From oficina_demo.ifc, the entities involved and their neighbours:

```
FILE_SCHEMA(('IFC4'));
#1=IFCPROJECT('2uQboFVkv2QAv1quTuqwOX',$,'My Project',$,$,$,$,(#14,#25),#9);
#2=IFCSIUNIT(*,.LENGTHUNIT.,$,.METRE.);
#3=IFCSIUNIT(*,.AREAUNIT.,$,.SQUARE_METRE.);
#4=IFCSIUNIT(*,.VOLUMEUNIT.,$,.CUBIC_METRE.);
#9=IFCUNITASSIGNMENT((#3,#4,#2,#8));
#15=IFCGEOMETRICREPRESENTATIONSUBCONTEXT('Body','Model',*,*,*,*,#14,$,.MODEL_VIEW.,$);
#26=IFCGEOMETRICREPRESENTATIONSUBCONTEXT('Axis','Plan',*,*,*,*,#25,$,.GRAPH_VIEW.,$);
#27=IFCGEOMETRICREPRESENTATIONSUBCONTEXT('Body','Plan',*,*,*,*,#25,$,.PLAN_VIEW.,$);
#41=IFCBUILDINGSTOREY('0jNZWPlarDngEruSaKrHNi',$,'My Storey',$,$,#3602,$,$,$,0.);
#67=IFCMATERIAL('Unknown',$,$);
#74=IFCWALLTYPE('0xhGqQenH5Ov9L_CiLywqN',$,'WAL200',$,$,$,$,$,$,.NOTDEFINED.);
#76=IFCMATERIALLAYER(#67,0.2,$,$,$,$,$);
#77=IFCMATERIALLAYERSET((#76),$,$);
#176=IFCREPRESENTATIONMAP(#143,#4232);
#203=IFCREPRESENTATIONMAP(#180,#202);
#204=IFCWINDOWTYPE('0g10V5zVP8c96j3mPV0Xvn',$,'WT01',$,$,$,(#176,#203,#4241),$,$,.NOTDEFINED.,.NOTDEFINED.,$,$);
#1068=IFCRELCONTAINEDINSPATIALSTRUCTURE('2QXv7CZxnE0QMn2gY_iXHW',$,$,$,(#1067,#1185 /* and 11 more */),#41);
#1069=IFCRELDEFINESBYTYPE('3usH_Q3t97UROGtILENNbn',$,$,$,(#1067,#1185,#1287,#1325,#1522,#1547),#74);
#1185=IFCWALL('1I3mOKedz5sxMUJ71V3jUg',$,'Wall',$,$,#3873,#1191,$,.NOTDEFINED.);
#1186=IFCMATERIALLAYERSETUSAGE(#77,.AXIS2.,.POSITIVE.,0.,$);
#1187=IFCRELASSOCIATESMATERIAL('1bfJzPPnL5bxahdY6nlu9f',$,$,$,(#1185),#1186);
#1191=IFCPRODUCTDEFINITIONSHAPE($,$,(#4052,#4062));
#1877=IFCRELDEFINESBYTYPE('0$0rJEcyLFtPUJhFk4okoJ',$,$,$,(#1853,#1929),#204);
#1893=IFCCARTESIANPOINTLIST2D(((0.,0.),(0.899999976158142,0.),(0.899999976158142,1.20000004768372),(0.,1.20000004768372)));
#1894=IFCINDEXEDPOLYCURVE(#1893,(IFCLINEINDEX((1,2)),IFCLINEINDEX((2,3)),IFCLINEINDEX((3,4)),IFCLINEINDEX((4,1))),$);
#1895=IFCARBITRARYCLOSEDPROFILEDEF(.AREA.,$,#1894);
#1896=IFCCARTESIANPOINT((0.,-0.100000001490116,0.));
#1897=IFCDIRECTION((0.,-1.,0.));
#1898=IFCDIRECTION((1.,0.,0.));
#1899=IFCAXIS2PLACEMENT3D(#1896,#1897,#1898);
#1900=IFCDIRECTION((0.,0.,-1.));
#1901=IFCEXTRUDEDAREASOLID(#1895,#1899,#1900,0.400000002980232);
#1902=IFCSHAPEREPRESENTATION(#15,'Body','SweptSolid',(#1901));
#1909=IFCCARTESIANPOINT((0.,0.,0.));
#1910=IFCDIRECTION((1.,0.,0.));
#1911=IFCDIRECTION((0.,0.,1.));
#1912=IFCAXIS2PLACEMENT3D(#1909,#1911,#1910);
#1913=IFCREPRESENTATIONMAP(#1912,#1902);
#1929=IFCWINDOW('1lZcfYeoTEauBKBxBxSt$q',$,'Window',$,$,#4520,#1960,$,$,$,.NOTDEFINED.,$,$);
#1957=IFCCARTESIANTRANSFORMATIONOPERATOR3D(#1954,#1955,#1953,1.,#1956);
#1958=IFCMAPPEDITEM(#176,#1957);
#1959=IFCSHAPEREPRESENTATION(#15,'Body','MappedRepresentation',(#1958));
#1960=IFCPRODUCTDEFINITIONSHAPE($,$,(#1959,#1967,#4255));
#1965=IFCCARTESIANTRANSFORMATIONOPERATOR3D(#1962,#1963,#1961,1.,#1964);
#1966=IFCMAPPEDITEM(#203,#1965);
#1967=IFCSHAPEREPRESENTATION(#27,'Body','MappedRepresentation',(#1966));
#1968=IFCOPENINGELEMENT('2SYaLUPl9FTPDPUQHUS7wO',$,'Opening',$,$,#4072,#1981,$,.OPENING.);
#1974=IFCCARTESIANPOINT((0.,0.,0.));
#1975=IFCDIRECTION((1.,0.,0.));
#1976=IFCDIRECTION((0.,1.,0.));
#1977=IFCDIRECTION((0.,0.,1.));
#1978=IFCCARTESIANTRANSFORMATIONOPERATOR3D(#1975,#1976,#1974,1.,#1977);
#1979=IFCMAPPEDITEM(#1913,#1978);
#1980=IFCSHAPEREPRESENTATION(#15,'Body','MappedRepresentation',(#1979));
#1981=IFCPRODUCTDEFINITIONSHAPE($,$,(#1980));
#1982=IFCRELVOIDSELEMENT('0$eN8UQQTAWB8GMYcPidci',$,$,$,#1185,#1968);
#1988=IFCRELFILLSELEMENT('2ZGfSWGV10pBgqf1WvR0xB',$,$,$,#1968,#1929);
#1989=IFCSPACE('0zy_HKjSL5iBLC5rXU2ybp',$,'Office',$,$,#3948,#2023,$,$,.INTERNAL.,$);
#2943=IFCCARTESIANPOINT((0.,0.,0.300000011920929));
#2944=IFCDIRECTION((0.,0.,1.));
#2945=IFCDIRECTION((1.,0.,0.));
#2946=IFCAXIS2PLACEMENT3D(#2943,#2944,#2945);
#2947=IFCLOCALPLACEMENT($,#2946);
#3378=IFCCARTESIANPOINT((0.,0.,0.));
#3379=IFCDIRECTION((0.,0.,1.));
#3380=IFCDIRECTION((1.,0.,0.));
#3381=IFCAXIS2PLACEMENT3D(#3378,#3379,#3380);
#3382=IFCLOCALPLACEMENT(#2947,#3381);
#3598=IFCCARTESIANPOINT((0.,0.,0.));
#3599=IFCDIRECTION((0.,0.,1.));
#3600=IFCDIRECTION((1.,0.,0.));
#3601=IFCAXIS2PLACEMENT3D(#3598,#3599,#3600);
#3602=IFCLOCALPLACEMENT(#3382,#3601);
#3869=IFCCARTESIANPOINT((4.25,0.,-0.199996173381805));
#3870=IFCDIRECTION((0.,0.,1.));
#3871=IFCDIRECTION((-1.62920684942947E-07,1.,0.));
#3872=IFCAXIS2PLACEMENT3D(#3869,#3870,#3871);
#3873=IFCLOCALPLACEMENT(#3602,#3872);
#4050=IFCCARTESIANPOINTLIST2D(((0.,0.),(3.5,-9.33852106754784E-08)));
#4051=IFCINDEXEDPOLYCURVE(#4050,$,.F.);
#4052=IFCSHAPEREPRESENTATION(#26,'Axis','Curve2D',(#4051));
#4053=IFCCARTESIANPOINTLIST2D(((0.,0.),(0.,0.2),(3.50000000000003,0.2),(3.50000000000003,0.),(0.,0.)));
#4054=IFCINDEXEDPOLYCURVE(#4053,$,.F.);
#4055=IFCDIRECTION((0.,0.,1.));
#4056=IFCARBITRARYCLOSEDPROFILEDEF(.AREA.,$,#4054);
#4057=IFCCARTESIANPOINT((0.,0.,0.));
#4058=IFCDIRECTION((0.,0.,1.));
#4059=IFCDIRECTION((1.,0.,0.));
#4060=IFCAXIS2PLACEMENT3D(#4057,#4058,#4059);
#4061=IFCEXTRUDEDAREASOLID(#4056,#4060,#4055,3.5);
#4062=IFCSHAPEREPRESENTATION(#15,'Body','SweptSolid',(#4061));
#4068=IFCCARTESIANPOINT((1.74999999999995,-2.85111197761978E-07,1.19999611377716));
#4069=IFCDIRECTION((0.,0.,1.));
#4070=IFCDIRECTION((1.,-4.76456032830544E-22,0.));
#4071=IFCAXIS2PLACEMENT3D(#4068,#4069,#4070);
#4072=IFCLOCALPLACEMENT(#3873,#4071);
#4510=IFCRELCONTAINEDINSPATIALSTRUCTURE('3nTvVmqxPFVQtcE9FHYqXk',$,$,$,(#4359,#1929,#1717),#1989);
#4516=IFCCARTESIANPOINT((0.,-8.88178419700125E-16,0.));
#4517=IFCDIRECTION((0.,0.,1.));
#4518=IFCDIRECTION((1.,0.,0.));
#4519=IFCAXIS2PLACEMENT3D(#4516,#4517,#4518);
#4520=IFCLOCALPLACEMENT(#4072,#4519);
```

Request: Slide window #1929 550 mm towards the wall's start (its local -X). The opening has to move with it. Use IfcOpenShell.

```python
import ifcopenshell
import ifcopenshell.api.geometry
import ifcopenshell.util.placement
import ifcopenshell.util.unit

model = ifcopenshell.open("oficina_demo.ifc")
unit_scale = ifcopenshell.util.unit.calculate_unit_scale(model)

window = model.by_guid("1lZcfYeoTEauBKBxBxSt$q")
opening = window.FillsVoids[0].RelatingOpeningElement
wall = opening.VoidsElements[0].RelatingBuildingElement

wall_matrix = ifcopenshell.util.placement.get_local_placement(wall.ObjectPlacement)
shift = wall_matrix[:3, 0] * -0.55 / unit_scale
before = ifcopenshell.util.placement.get_local_placement(window.ObjectPlacement)[:3, 3].copy()

# The window is placed relative to its opening, so it follows when the opening moves.
matrix = ifcopenshell.util.placement.get_local_placement(opening.ObjectPlacement)
matrix[:3, 3] += shift
ifcopenshell.api.geometry.edit_object_placement(
    model, product=opening, matrix=matrix, is_si=False, should_transform_children=True
)

after = ifcopenshell.util.placement.get_local_placement(window.ObjectPlacement)[:3, 3]
print("window moved by", (after - before).round(3) + 0.0)

model.write("oficina_demo_rev.ifc")
```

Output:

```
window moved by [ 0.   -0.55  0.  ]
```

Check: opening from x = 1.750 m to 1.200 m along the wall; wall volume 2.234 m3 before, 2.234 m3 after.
